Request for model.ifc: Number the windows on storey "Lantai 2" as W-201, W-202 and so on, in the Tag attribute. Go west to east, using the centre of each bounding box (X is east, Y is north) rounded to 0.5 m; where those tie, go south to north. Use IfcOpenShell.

First a look at what the model holds.

```python
import ifcopenshell
import ifcopenshell.util.element
import ifcopenshell.util.placement

model = ifcopenshell.open("model.ifc")
print(model.schema)
storey = next(s for s in model.by_type("IfcBuildingStorey") if s.Name == "Lantai 2")
windows = [e for e in ifcopenshell.util.element.get_decomposition(storey) if e.is_a("IfcWindow")]
for e in sorted(windows, key=lambda e: e.id()):
    origin = ifcopenshell.util.placement.get_local_placement(e.ObjectPlacement)[:3, 3]
    print(e.id(), e.Tag, e.Name, origin.round(2) + 0.0, sep=" | ")
```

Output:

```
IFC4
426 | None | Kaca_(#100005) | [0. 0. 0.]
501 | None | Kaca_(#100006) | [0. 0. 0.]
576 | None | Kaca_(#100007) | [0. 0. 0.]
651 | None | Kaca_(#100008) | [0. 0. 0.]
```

```python
import ifcopenshell
import ifcopenshell.geom
import ifcopenshell.util.element
import ifcopenshell.util.shape

model = ifcopenshell.open("model.ifc")
settings = ifcopenshell.geom.settings()
settings.set("use-world-coords", True)


def centre(element):
    shape = ifcopenshell.geom.create_shape(settings, element)
    return ifcopenshell.util.shape.get_bbox_centroid(shape.geometry)


storey = next(s for s in model.by_type("IfcBuildingStorey") if s.Name == "Lantai 2")
windows = [e for e in ifcopenshell.util.element.get_decomposition(storey) if e.is_a("IfcWindow")]

# Insertion points can sit at a corner or the storey origin, so sort by the geometry (in metres).
centres = {e: centre(e) for e in windows}
windows.sort(key=lambda e: (round(centres[e][0] / 0.5), centres[e][1]))

for i, e in enumerate(windows, start=1):
    number = f"W-2{i:02d}"
    e.Tag = number
    print(e.id(), number)

model.write("model_v2.ifc")
```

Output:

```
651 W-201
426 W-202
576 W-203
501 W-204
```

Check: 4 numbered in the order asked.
